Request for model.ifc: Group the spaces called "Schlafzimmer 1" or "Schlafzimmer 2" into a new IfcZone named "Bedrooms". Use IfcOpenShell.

First a look at what the model holds.

```python
import ifcopenshell

model = ifcopenshell.open("model.ifc")
print(model.schema)
seen = {}
for space in model.by_type("IfcSpace"):
    seen[space.LongName] = seen.get(space.LongName, 0) + 1
for name, count in sorted(seen.items(), key=str):
    print(count, "x", name)
print("zones:", [z.Name for z in model.by_type("IfcZone")][:20])
```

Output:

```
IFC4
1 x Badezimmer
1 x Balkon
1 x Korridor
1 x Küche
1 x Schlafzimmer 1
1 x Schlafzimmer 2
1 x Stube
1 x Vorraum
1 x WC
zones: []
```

```python
import ifcopenshell
import ifcopenshell.api.group
import ifcopenshell.api.root

model = ifcopenshell.open("model.ifc")

names = {"Schlafzimmer 1", "Schlafzimmer 2"}
spaces = [s for s in model.by_type("IfcSpace") if s.LongName in names]

zone = ifcopenshell.api.root.create_entity(model, ifc_class="IfcZone", name="Bedrooms")
ifcopenshell.api.group.assign_group(model, products=spaces, group=zone)
print(len(spaces), "spaces in", zone.Name)

model.write("model_v2.ifc")
```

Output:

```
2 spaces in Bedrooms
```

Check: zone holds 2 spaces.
